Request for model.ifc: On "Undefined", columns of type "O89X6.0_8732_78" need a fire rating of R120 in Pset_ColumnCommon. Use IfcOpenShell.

First a look at what the model holds.

```python
import ifcopenshell
import ifcopenshell.util.element

model = ifcopenshell.open("model.ifc")
print(model.schema)
storey = next(s for s in model.by_type("IfcBuildingStorey") if s.Name == "Undefined")
columns = [e for e in ifcopenshell.util.element.get_decomposition(storey) if e.is_a("IfcColumn")]
seen = {}
for e in columns:
    element_type = ifcopenshell.util.element.get_type(e)
    key = (element_type.Name if element_type != e and element_type else None, ifcopenshell.util.element.get_pset(e, "Pset_ColumnCommon", "FireRating"))
    seen[key] = seen.get(key, 0) + 1
for (name, value), count in sorted(seen.items(), key=str):
    print(count, "x", name, "|", value)
```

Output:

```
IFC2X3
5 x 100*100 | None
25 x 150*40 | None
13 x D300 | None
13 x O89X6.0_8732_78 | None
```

```python
import ifcopenshell
import ifcopenshell.api.pset
import ifcopenshell.util.element

model = ifcopenshell.open("model.ifc")

storey = next(s for s in model.by_type("IfcBuildingStorey") if s.Name == "Undefined")
columns = [e for e in ifcopenshell.util.element.get_decomposition(storey) if e.is_a("IfcColumn")]

count = 0
for e in columns:
    element_type = ifcopenshell.util.element.get_type(e)
    if element_type in (None, e) or element_type.Name != "O89X6.0_8732_78":
        continue
    found = ifcopenshell.util.element.get_pset(e, "Pset_ColumnCommon", should_inherit=False)
    if found:
        pset = model.by_id(found["id"])
        if len(ifcopenshell.util.element.get_elements_by_pset(pset)) > 1:
            pset = ifcopenshell.api.pset.unshare_pset(model, products=[e], pset=pset)[0]
    else:
        pset = ifcopenshell.api.pset.add_pset(model, product=e, name="Pset_ColumnCommon")
    ifcopenshell.api.pset.edit_pset(model, pset=pset, properties={"FireRating": "R120"})
    count += 1

print(count, "columns updated")

model.write("model_rev.ifc")
```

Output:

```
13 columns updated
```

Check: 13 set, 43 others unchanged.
